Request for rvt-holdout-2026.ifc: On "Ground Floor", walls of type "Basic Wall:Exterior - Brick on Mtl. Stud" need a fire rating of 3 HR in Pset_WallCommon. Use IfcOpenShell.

First a look at what the model holds.

```python
import ifcopenshell
import ifcopenshell.util.element

model = ifcopenshell.open("rvt-holdout-2026.ifc")
print(model.schema)
storey = next(s for s in model.by_type("IfcBuildingStorey") if s.Name == "Ground Floor")
walls = [e for e in ifcopenshell.util.element.get_decomposition(storey) if e.is_a("IfcWall")]
seen = {}
for e in walls:
    element_type = ifcopenshell.util.element.get_type(e)
    key = (element_type.Name if element_type != e and element_type else None, ifcopenshell.util.element.get_pset(e, "Pset_WallCommon", "FireRating"))
    seen[key] = seen.get(key, 0) + 1
for (name, value), count in sorted(seen.items(), key=str):
    print(count, "x", name, "|", value)
```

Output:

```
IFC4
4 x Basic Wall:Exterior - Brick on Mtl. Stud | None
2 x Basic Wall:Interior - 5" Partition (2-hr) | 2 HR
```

```python
import ifcopenshell
import ifcopenshell.api.pset
import ifcopenshell.util.element

model = ifcopenshell.open("rvt-holdout-2026.ifc")

storey = next(s for s in model.by_type("IfcBuildingStorey") if s.Name == "Ground Floor")
walls = [e for e in ifcopenshell.util.element.get_decomposition(storey) if e.is_a("IfcWall")]

count = 0
for e in walls:
    element_type = ifcopenshell.util.element.get_type(e)
    if element_type in (None, e) or element_type.Name != "Basic Wall:Exterior - Brick on Mtl. Stud":
        continue
    # add_pset returns the element's existing set when there is one.
    pset = ifcopenshell.api.pset.add_pset(model, product=e, name="Pset_WallCommon")
    ifcopenshell.api.pset.edit_pset(model, pset=pset, properties={"FireRating": "3 HR"})
    count += 1

print(count, "walls updated")

model.write("rvt-holdout-2026_v2.ifc")
```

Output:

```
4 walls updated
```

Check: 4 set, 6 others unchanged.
